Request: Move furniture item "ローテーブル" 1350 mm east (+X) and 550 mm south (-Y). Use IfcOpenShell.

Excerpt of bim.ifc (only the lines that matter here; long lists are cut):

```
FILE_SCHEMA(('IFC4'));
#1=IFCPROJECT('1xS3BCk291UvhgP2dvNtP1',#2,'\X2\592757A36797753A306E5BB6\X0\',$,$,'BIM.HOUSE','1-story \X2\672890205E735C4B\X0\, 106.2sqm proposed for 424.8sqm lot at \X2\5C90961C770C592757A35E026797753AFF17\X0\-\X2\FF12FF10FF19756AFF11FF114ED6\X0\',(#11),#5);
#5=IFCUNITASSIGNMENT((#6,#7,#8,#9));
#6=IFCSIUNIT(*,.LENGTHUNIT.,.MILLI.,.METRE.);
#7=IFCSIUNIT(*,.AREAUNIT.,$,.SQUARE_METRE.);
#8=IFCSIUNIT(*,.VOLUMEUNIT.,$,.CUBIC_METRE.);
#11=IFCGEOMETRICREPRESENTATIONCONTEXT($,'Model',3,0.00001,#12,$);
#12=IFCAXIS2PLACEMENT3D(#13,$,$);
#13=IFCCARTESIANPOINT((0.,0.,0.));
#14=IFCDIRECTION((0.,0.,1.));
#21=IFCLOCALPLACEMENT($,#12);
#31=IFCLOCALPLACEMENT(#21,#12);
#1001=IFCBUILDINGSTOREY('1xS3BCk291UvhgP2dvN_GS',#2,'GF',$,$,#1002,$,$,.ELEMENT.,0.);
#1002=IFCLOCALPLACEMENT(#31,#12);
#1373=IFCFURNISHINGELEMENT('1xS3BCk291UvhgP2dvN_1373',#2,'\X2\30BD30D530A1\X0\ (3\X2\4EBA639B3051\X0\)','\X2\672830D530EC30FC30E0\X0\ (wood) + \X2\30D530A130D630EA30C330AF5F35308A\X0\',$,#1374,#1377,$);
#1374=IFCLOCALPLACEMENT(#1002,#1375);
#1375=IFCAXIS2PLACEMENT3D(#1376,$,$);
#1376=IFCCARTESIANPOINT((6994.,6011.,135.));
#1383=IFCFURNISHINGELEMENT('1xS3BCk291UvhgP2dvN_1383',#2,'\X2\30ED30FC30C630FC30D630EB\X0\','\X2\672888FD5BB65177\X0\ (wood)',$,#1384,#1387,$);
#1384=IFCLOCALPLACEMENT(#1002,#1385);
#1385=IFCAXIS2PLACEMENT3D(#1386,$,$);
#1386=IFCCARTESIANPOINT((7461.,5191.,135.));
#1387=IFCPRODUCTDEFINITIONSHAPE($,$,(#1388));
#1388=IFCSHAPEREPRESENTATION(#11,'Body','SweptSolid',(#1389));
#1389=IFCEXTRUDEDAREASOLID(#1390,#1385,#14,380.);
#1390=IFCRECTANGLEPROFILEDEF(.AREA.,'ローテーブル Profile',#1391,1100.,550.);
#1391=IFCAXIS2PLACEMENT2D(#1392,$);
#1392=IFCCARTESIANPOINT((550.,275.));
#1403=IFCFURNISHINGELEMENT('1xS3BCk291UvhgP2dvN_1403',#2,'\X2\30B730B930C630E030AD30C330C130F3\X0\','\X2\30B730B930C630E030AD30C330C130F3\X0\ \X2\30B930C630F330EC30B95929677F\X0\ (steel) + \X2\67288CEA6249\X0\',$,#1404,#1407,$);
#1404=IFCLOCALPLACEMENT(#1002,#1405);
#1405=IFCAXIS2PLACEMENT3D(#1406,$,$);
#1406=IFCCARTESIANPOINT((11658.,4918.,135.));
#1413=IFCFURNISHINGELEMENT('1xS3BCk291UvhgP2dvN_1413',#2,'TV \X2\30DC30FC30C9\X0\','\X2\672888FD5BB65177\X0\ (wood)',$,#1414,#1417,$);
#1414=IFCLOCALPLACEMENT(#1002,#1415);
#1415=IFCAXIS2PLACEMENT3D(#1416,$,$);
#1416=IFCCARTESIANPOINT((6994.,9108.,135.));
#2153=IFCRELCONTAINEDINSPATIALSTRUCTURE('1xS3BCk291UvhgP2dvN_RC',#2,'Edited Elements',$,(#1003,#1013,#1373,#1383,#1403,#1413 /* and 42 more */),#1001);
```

```python
import ifcopenshell
import ifcopenshell.api.geometry
import ifcopenshell.util.placement

model = ifcopenshell.open("bim.ifc")

item = model.by_guid("1xS3BCk291UvhgP2dvN_1383")
matrix = ifcopenshell.util.placement.get_local_placement(item.ObjectPlacement)
matrix[0, 3] += 1350.0
matrix[1, 3] -= 550.0
ifcopenshell.api.geometry.edit_object_placement(model, product=item, matrix=matrix, is_si=False)

print(ifcopenshell.util.placement.get_local_placement(item.ObjectPlacement).round(3) + 0.0)

model.write("bim_v2.ifc")
```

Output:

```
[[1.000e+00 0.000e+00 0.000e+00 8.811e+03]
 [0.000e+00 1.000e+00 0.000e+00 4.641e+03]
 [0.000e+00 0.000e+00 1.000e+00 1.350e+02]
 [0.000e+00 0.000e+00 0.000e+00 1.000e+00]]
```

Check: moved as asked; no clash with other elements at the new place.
